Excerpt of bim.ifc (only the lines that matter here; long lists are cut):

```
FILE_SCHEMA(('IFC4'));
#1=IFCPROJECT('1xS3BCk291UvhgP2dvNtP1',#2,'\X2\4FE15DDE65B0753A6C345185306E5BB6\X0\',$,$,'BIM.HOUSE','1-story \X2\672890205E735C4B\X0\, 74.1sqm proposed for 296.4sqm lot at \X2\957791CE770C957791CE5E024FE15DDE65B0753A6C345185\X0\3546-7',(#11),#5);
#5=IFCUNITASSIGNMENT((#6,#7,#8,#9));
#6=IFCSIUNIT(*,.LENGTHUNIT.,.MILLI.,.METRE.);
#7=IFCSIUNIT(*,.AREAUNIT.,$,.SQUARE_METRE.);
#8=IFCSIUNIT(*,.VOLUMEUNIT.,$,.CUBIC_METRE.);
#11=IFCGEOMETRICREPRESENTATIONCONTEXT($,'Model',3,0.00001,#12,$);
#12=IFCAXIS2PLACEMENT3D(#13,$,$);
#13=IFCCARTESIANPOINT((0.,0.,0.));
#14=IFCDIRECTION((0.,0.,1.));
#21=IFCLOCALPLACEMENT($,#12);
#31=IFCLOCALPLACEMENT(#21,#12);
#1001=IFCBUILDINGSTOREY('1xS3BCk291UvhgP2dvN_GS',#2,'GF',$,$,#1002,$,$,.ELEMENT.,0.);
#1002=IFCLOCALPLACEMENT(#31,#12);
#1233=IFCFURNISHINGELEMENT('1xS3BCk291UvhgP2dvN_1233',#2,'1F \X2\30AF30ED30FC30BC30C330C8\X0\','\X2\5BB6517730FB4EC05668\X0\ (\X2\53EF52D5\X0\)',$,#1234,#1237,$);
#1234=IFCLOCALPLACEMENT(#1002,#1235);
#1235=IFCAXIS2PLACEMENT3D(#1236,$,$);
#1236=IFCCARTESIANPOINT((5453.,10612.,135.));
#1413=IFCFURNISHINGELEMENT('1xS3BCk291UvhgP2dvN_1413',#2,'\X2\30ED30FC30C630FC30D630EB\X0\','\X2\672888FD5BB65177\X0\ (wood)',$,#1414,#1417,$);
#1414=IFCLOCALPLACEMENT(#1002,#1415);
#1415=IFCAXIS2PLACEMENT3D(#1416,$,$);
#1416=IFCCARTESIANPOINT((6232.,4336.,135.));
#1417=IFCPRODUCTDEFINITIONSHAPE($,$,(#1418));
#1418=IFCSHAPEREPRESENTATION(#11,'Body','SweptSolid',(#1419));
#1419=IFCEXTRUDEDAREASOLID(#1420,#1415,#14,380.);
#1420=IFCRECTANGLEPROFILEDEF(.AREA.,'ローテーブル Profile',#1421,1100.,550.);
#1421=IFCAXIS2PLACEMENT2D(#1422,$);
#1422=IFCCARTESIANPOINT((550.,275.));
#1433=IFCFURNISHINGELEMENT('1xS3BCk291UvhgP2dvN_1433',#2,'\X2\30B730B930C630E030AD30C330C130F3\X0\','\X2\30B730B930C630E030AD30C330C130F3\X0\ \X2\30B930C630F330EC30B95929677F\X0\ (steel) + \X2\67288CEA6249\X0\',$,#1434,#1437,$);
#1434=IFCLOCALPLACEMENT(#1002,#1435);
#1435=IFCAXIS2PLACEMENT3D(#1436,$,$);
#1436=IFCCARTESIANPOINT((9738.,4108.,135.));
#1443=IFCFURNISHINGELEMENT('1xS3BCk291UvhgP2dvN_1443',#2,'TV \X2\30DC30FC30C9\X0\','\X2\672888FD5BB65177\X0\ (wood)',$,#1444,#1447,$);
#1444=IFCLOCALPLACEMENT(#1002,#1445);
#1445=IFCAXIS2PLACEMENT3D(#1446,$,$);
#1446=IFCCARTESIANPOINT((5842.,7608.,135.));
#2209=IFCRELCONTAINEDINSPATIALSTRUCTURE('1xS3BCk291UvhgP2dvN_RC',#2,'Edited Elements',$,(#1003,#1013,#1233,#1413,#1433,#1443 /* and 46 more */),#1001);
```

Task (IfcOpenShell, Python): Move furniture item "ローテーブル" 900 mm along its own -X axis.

```python
import ifcopenshell
import ifcopenshell.api.geometry
import ifcopenshell.util.placement

model = ifcopenshell.open("bim.ifc")

item = model.by_guid("1xS3BCk291UvhgP2dvN_1413")
matrix = ifcopenshell.util.placement.get_local_placement(item.ObjectPlacement)
matrix[:3, 3] -= matrix[:3, 0] * 900.0
ifcopenshell.api.geometry.edit_object_placement(model, product=item, matrix=matrix, is_si=False)

print(ifcopenshell.util.placement.get_local_placement(item.ObjectPlacement).round(3) + 0.0)

model.write("bim_v2.ifc")
```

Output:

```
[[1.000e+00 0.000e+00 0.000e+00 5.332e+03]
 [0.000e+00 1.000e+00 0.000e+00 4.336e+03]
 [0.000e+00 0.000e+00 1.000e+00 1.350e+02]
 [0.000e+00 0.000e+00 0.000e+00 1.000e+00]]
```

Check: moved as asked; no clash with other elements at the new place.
